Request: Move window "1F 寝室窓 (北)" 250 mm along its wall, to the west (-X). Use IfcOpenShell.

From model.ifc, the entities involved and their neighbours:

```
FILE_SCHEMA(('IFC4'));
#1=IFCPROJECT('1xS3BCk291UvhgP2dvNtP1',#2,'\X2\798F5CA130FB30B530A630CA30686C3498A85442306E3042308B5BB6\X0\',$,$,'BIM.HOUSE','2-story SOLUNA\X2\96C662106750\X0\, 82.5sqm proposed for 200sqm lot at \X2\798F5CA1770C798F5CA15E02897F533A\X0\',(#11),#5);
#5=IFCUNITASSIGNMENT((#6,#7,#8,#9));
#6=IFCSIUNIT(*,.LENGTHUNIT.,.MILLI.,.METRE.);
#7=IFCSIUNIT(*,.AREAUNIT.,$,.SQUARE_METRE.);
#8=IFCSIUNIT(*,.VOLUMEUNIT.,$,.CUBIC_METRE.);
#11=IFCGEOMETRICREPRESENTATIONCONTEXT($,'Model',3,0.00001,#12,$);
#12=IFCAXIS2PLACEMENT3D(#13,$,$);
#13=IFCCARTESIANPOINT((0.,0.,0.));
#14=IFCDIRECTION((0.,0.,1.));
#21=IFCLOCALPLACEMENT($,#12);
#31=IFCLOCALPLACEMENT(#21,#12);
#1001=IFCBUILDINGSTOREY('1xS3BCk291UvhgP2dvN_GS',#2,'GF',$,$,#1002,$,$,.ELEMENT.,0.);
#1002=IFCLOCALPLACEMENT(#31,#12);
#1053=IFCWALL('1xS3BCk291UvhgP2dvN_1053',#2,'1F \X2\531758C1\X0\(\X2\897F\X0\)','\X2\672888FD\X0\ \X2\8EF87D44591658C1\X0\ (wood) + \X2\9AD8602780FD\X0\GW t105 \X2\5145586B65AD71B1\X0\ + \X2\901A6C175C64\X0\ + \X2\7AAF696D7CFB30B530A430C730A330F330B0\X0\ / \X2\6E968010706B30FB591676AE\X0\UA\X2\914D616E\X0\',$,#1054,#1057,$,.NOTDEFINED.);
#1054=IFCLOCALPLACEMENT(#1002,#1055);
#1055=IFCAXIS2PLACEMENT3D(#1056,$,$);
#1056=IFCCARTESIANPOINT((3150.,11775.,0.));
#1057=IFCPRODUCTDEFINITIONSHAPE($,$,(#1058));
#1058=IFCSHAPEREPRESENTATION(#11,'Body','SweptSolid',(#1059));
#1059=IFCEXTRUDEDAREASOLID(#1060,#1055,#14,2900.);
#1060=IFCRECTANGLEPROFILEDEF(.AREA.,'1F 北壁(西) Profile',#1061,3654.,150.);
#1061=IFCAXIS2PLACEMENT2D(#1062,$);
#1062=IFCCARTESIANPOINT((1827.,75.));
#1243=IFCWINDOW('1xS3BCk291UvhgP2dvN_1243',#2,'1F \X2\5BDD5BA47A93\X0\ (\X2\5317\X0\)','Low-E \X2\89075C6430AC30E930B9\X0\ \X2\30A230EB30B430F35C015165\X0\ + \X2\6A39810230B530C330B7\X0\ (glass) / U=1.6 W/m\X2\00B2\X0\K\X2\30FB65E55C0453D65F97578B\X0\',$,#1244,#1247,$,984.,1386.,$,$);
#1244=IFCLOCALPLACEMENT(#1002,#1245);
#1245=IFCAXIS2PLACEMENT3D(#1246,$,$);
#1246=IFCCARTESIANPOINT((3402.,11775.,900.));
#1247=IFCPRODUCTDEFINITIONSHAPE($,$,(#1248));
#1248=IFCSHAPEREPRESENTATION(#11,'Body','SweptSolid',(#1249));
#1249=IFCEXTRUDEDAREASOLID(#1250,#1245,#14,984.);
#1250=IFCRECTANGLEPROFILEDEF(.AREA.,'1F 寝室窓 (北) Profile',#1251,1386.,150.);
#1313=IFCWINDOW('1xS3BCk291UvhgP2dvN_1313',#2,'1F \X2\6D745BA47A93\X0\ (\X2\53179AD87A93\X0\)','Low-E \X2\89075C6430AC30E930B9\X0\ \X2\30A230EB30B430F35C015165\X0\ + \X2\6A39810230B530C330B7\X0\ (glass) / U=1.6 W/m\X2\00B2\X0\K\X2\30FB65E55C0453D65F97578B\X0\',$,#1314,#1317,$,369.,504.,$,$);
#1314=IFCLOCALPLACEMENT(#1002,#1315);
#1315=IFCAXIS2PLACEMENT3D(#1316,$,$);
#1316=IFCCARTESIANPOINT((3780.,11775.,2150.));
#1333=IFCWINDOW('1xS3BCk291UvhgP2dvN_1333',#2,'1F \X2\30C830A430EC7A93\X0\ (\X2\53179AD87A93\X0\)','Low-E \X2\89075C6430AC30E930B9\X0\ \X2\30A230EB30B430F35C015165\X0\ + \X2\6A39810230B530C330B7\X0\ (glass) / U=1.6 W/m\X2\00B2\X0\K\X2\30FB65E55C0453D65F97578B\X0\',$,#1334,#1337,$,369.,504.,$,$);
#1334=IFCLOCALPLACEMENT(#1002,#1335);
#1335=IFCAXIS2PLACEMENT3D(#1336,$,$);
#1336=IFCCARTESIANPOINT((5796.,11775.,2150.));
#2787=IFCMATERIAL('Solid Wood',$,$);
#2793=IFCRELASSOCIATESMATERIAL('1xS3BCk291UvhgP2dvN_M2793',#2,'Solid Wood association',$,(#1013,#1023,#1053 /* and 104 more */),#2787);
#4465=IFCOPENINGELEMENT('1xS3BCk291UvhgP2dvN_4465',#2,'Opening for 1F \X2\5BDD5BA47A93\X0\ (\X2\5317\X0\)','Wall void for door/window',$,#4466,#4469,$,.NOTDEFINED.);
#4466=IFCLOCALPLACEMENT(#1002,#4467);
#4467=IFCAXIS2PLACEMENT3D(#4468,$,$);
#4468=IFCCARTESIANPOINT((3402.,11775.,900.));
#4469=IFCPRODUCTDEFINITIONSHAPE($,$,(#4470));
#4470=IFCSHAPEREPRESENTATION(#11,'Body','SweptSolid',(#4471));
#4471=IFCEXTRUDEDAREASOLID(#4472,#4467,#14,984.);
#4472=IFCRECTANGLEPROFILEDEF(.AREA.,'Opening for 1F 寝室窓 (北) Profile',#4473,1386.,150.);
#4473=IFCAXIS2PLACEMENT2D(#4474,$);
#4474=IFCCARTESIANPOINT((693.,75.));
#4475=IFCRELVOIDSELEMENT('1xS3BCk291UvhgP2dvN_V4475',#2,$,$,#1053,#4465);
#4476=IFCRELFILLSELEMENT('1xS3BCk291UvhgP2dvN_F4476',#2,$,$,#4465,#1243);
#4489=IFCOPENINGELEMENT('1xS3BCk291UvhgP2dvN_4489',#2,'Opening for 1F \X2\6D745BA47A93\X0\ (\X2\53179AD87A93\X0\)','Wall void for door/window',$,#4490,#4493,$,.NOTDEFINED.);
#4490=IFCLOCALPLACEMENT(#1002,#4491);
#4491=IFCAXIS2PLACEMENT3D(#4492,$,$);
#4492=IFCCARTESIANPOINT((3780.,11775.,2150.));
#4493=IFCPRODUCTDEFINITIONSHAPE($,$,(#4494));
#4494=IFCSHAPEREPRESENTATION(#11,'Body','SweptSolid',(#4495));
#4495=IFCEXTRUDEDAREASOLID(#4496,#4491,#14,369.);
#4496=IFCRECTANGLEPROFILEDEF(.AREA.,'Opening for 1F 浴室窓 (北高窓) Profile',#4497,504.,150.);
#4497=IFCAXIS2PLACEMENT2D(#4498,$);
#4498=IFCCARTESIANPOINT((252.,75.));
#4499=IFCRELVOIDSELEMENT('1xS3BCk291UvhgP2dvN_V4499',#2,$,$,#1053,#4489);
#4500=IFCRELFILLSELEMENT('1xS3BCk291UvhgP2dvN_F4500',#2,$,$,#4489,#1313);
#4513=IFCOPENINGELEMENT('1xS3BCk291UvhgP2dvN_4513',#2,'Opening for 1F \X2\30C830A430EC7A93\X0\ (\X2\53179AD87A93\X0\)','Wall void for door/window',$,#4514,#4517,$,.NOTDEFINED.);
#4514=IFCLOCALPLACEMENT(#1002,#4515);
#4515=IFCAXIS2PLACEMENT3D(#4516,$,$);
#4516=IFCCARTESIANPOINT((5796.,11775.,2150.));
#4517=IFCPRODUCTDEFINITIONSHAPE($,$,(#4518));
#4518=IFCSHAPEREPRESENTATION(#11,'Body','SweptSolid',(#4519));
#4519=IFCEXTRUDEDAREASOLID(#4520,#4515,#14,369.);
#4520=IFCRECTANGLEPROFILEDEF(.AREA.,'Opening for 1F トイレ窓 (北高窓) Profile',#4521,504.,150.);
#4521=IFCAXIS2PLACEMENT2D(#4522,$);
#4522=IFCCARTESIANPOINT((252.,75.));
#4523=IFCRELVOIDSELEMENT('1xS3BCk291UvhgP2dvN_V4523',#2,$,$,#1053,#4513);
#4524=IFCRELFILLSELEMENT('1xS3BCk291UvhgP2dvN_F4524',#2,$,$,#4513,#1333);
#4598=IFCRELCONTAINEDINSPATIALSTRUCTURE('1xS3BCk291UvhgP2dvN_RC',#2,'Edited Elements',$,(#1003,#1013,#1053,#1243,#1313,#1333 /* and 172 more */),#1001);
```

```python
import ifcopenshell
import ifcopenshell.api.geometry
import ifcopenshell.util.placement

model = ifcopenshell.open("model.ifc")

window = model.by_id(1243)
opening = window.FillsVoids[0].RelatingOpeningElement
wall = opening.VoidsElements[0].RelatingBuildingElement

wall_matrix = ifcopenshell.util.placement.get_local_placement(wall.ObjectPlacement)
shift = wall_matrix[:3, 0] * -250.0
before = ifcopenshell.util.placement.get_local_placement(window.ObjectPlacement)[:3, 3].copy()

# The window is not placed relative to its opening, so move both.
for product in (opening, window):
    matrix = ifcopenshell.util.placement.get_local_placement(product.ObjectPlacement)
    matrix[:3, 3] += shift
    ifcopenshell.api.geometry.edit_object_placement(model, product=product, matrix=matrix, is_si=False)

after = ifcopenshell.util.placement.get_local_placement(window.ObjectPlacement)[:3, 3]
print("window moved by", (after - before).round(3) + 0.0)

model.write("model_updated.ifc")
```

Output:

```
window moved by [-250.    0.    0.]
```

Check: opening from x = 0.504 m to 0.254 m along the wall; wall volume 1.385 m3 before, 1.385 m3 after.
